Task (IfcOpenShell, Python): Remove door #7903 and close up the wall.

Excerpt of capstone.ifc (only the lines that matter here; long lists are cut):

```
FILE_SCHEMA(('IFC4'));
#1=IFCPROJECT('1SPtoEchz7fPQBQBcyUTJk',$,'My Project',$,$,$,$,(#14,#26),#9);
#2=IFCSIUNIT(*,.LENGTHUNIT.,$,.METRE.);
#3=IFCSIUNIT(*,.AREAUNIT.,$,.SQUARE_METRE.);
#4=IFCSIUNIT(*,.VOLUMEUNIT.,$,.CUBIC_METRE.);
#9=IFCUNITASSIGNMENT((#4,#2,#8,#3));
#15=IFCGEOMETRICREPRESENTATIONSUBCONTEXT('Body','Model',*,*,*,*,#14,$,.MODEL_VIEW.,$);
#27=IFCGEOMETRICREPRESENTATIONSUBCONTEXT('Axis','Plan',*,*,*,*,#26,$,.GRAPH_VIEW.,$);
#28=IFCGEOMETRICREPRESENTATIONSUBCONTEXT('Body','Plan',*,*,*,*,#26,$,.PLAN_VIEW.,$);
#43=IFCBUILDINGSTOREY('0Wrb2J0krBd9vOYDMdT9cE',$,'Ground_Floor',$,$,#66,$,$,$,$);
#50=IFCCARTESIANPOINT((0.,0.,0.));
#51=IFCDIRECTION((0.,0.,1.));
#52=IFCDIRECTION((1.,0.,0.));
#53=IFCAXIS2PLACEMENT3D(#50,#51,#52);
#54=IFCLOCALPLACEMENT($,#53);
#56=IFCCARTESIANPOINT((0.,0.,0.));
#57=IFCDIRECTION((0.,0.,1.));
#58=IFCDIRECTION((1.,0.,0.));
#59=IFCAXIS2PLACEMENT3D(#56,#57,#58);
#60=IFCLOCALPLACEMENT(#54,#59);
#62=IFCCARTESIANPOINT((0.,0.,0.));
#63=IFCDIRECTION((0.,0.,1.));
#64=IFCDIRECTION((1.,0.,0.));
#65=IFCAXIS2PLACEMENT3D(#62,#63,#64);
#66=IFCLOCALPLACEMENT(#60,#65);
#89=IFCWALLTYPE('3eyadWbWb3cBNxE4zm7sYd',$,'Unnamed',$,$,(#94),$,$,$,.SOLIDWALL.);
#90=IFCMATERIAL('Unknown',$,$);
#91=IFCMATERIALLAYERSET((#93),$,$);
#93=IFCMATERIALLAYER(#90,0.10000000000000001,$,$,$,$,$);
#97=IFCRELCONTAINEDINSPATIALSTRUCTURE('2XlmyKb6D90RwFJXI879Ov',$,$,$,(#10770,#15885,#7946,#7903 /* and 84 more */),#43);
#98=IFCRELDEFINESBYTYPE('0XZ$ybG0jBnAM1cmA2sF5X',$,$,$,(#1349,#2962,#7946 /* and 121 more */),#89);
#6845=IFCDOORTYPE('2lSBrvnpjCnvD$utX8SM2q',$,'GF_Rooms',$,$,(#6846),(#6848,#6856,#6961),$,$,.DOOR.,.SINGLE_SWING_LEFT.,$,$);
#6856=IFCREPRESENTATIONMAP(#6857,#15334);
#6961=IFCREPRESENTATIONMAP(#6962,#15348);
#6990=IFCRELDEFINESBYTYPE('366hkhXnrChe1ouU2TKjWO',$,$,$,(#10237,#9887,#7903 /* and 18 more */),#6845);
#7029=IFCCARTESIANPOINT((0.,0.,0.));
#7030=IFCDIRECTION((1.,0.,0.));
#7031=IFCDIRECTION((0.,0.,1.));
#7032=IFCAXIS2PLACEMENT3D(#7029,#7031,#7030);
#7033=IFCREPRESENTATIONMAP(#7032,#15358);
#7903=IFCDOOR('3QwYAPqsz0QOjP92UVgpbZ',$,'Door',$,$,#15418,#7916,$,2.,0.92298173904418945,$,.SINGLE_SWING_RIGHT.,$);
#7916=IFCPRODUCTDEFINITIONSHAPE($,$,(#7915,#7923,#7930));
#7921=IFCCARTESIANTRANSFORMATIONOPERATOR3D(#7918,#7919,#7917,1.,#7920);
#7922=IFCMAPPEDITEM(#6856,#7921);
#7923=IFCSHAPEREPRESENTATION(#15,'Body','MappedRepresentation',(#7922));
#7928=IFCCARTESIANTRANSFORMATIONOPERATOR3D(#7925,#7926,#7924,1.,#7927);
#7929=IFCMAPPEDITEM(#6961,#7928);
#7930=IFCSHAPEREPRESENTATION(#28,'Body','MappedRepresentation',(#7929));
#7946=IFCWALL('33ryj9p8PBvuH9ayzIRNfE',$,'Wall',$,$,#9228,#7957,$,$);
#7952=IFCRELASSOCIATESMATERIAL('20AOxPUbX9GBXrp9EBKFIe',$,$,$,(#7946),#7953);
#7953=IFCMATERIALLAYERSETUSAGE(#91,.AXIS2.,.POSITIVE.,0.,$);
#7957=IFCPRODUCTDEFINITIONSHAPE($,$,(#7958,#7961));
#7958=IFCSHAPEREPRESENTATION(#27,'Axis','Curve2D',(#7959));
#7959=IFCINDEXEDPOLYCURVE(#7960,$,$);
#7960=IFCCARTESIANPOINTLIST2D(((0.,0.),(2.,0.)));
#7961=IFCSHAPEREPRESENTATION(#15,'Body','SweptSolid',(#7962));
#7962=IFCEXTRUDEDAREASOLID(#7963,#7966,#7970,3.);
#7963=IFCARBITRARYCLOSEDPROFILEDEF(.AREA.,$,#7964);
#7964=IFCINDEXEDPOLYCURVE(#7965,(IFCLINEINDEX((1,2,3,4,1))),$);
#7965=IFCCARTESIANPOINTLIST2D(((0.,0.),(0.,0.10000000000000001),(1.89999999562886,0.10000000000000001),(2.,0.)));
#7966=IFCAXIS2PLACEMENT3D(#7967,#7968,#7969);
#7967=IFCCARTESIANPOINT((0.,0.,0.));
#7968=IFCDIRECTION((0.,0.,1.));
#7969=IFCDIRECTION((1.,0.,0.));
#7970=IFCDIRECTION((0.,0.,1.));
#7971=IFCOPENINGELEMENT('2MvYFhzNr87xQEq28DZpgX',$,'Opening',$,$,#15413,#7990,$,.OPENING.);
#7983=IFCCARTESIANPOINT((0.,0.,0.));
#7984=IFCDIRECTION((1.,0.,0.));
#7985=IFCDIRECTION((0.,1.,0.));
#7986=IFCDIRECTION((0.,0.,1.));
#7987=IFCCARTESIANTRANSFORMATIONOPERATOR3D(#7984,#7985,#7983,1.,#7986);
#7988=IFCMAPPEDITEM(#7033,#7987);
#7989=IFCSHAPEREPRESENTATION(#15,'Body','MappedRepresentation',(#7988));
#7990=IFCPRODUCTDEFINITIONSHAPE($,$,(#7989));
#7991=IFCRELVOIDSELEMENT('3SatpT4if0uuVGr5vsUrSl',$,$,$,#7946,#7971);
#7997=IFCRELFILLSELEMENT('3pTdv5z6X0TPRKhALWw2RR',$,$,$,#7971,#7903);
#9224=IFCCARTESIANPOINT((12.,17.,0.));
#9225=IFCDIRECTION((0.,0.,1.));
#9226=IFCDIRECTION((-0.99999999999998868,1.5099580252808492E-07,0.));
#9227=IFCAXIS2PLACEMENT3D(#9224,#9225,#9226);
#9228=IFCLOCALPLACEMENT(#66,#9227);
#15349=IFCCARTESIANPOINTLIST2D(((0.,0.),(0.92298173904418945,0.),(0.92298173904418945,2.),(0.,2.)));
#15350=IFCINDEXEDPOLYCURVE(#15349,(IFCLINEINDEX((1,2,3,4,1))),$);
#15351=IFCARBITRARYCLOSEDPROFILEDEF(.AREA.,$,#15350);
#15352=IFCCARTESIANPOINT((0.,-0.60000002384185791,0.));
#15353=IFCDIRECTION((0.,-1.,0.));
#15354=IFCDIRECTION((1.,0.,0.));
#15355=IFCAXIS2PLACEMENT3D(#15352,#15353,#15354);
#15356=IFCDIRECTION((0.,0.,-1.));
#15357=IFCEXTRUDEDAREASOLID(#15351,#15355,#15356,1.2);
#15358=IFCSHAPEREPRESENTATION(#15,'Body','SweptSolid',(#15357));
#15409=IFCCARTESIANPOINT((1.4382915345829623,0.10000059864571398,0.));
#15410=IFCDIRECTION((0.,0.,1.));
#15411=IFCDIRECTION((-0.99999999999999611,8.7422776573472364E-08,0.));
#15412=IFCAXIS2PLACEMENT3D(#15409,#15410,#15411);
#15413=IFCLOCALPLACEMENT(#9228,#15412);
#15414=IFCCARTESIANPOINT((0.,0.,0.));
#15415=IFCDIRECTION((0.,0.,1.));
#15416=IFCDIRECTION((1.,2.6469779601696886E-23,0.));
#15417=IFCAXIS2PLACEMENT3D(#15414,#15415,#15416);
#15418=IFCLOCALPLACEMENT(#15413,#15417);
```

```python
import ifcopenshell
import ifcopenshell.api.feature
import ifcopenshell.api.root
import ifcopenshell.geom
import ifcopenshell.util.shape

model = ifcopenshell.open("capstone.ifc")
settings = ifcopenshell.geom.settings()


def volume(element):
    """Net volume in cubic metres, openings subtracted."""
    shape = ifcopenshell.geom.create_shape(settings, element)
    return ifcopenshell.util.shape.get_volume(shape.geometry)


door = model.by_guid("3QwYAPqsz0QOjP92UVgpbZ")
opening = door.FillsVoids[0].RelatingOpeningElement
wall = opening.VoidsElements[0].RelatingBuildingElement
before = volume(wall)

ifcopenshell.api.root.remove_product(model, product=door)
ifcopenshell.api.feature.remove_feature(model, feature=opening)

after = volume(wall)

print(f"wall volume {before:.3f} -> {after:.3f} m3")

model.write("capstone_v2.ifc")
```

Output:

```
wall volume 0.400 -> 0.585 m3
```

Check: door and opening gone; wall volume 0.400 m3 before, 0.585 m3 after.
